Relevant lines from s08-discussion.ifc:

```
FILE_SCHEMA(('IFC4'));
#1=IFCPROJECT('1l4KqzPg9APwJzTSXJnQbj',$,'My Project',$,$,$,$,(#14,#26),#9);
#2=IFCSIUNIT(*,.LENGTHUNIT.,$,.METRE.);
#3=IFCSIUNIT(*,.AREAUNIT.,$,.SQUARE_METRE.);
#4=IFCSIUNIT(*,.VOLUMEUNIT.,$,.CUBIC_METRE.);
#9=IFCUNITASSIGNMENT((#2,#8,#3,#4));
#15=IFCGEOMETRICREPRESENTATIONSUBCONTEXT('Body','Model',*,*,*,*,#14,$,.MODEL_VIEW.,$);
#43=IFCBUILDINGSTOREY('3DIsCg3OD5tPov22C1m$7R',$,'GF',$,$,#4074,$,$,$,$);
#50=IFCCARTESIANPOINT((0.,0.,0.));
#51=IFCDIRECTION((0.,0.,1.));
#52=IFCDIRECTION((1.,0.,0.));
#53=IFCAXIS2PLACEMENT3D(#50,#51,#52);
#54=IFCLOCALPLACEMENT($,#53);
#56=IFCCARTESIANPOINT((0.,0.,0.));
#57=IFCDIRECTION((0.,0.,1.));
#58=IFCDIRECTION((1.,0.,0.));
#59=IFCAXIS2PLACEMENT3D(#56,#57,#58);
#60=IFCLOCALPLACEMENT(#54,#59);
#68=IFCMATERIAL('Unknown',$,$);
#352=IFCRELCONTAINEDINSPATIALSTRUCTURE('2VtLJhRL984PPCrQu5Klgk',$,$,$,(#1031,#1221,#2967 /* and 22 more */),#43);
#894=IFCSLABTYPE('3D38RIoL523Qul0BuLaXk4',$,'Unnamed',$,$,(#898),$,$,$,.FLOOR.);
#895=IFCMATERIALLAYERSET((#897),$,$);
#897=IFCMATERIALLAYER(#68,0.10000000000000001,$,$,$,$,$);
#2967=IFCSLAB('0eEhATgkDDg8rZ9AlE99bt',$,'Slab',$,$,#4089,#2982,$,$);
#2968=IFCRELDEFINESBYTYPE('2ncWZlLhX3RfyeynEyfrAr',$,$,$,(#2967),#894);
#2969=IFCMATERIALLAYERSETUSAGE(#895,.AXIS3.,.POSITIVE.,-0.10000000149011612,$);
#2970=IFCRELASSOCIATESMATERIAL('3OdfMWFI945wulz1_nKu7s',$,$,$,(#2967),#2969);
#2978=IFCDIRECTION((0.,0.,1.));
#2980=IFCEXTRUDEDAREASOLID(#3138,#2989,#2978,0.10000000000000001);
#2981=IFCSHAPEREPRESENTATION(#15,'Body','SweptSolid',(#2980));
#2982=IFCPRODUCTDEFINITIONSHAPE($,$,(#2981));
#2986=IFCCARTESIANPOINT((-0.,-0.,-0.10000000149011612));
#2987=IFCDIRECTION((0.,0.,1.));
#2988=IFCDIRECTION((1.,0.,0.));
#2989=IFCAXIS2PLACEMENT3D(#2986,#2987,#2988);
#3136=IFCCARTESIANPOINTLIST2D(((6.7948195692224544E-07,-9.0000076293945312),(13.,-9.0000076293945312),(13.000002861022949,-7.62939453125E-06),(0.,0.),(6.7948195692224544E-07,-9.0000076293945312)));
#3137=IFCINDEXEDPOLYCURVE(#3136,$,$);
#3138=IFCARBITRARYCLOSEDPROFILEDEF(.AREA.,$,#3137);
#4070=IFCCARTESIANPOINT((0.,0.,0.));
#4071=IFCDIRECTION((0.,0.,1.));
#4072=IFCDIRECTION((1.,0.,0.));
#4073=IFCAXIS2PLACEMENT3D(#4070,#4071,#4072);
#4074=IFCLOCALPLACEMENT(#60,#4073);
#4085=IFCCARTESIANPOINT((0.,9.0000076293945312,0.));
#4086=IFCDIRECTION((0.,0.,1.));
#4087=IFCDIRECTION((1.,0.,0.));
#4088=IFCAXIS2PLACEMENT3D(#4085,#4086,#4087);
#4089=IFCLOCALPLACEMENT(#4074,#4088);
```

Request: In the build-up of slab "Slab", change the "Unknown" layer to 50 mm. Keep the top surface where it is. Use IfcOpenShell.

```python
import ifcopenshell
import ifcopenshell.util.element
import ifcopenshell.util.representation
import ifcopenshell.util.unit

model = ifcopenshell.open("s08-discussion.ifc")
unit_scale = ifcopenshell.util.unit.calculate_unit_scale(model)

layer_set = model.by_id(895)
layer = next(l for l in layer_set.MaterialLayers if l.Material and l.Material.Name == "Unknown")
change = 0.05 / unit_scale - layer.LayerThickness
layer.LayerThickness += change

# Geometry does not follow the layer set by itself.
slabs = [e for e in ifcopenshell.util.element.get_elements_by_material(model, layer_set) if e.is_a("IfcSlab")]
for slab in sorted(slabs, key=lambda e: e.id()):
    body = ifcopenshell.util.representation.get_representation(slab, "Model", "Body")
    solid = body.Items[0]
    old_depth = solid.Depth
    solid.Depth += change
    # Extruded upwards: lower the start of the extrusion so the top stays.
    x, y, z = solid.Position.Location.Coordinates
    solid.Position.Location = model.createIfcCartesianPoint((x, y, z - change))
    print(slab.id(), f"{old_depth:g} -> {solid.Depth:g}")

# The layers are counted up from the underside, which has moved.
for usage in {ifcopenshell.util.element.get_material(slab) for slab in slabs}:
    usage.OffsetFromReferenceLine -= change

model.write("s08-discussion_edited.ifc")
```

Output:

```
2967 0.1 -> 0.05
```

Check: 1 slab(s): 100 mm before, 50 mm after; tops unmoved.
